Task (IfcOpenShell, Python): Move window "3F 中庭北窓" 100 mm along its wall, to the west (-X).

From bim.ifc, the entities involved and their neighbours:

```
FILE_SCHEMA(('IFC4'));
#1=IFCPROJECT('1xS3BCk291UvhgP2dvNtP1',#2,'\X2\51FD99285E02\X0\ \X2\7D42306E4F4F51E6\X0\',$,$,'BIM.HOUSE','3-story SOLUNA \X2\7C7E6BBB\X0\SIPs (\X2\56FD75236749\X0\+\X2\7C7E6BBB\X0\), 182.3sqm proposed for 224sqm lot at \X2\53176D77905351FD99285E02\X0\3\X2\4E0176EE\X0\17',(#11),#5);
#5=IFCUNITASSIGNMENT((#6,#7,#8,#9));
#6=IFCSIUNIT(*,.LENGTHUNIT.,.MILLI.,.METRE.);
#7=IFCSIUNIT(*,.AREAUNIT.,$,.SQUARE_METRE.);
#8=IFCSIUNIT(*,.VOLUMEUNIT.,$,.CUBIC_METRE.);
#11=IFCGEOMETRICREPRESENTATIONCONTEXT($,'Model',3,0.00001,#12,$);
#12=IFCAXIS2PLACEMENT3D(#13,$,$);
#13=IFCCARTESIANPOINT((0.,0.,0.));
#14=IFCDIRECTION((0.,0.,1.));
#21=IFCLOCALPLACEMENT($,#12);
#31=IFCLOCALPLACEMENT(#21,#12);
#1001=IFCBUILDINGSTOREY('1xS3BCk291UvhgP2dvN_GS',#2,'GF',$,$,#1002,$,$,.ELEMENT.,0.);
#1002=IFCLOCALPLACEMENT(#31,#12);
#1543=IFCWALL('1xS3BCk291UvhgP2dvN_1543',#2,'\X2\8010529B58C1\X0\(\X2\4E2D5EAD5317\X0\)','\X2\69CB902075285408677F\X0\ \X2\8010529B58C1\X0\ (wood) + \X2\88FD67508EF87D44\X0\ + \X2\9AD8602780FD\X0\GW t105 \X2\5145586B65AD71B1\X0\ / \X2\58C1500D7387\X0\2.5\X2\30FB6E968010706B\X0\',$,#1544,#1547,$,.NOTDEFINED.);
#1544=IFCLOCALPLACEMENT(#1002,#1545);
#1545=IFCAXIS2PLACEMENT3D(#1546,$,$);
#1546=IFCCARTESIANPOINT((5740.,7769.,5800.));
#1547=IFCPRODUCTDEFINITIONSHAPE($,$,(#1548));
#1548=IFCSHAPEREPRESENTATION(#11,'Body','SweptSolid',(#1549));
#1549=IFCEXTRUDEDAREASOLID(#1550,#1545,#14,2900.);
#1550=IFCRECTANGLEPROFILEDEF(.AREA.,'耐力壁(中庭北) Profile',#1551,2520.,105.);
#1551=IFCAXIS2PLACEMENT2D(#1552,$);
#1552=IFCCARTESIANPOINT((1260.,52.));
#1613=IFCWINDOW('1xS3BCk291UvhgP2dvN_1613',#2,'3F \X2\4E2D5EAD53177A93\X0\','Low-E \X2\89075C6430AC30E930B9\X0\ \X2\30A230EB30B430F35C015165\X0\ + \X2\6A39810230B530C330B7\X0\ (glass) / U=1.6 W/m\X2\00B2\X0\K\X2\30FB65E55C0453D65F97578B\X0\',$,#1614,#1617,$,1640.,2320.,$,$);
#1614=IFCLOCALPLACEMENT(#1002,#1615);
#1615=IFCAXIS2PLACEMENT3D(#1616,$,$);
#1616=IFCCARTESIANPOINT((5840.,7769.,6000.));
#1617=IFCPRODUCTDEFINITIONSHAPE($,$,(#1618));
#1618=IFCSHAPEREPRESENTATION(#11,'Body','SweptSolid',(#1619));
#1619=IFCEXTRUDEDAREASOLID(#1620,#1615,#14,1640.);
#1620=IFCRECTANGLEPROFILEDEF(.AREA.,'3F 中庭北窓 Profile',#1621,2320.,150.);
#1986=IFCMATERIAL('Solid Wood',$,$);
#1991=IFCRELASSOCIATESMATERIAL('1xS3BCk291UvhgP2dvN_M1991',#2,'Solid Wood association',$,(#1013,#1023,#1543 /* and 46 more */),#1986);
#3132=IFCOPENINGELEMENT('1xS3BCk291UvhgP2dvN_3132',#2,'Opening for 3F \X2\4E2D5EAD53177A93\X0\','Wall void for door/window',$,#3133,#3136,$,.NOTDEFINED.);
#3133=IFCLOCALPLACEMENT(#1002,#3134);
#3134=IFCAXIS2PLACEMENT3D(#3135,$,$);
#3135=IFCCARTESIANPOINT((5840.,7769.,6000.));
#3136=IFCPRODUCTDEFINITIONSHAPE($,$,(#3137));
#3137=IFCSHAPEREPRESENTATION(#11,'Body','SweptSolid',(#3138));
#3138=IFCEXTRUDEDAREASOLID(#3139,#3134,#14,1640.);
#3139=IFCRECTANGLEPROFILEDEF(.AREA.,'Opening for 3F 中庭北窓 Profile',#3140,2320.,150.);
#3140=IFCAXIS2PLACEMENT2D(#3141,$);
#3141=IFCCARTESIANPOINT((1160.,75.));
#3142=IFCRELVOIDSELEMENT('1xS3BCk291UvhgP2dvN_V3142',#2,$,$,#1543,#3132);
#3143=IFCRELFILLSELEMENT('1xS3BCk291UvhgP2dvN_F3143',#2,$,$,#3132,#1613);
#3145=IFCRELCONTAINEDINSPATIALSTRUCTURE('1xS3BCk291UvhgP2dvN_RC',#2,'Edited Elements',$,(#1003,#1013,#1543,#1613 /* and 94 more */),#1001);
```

```python
import ifcopenshell
import ifcopenshell.api.geometry
import ifcopenshell.util.placement
import ifcopenshell.util.unit

model = ifcopenshell.open("bim.ifc")
unit_scale = ifcopenshell.util.unit.calculate_unit_scale(model)

window = model.by_guid("1xS3BCk291UvhgP2dvN_1613")
opening = window.FillsVoids[0].RelatingOpeningElement
wall = opening.VoidsElements[0].RelatingBuildingElement

wall_matrix = ifcopenshell.util.placement.get_local_placement(wall.ObjectPlacement)
shift = wall_matrix[:3, 0] * -0.1 / unit_scale
before = ifcopenshell.util.placement.get_local_placement(window.ObjectPlacement)[:3, 3].copy()

# The window is not placed relative to its opening, so move both.
for product in (opening, window):
    matrix = ifcopenshell.util.placement.get_local_placement(product.ObjectPlacement)
    matrix[:3, 3] += shift
    ifcopenshell.api.geometry.edit_object_placement(model, product=product, matrix=matrix, is_si=False)

after = ifcopenshell.util.placement.get_local_placement(window.ObjectPlacement)[:3, 3]
print("window moved by", (after - before).round(3) + 0.0)

model.write("bim_rev.ifc")
```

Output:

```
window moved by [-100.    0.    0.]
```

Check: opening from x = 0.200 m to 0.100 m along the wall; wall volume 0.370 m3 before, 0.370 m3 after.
